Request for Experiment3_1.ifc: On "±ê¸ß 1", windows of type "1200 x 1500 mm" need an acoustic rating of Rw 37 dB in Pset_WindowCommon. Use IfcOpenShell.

First a look at what the model holds.

```python
import ifcopenshell
import ifcopenshell.util.element

model = ifcopenshell.open("Experiment3_1.ifc")
print(model.schema)
storey = next(s for s in model.by_type("IfcBuildingStorey") if s.Name == "±ê¸ß 1")
windows = [e for e in ifcopenshell.util.element.get_decomposition(storey) if e.is_a("IfcWindow")]
seen = {}
for e in windows:
    element_type = ifcopenshell.util.element.get_type(e)
    key = (element_type.Name if element_type != e and element_type else None, ifcopenshell.util.element.get_pset(e, "Pset_WindowCommon", "AcousticRating"))
    seen[key] = seen.get(key, 0) + 1
for (name, value), count in sorted(seen.items(), key=str):
    print(count, "x", name, "|", value)
```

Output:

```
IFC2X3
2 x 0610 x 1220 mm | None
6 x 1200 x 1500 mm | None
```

```python
import ifcopenshell
import ifcopenshell.api.pset
import ifcopenshell.util.element

model = ifcopenshell.open("Experiment3_1.ifc")

storey = next(s for s in model.by_type("IfcBuildingStorey") if s.Name == "±ê¸ß 1")
windows = [e for e in ifcopenshell.util.element.get_decomposition(storey) if e.is_a("IfcWindow")]

count = 0
for e in windows:
    element_type = ifcopenshell.util.element.get_type(e)
    if element_type in (None, e) or element_type.Name != "1200 x 1500 mm":
        continue
    # add_pset returns the element's existing set when there is one.
    pset = ifcopenshell.api.pset.add_pset(model, product=e, name="Pset_WindowCommon")
    ifcopenshell.api.pset.edit_pset(model, pset=pset, properties={"AcousticRating": "Rw 37 dB"})
    count += 1

print(count, "windows updated")

model.write("Experiment3_1_rev.ifc")
```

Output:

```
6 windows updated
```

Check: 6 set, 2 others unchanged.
